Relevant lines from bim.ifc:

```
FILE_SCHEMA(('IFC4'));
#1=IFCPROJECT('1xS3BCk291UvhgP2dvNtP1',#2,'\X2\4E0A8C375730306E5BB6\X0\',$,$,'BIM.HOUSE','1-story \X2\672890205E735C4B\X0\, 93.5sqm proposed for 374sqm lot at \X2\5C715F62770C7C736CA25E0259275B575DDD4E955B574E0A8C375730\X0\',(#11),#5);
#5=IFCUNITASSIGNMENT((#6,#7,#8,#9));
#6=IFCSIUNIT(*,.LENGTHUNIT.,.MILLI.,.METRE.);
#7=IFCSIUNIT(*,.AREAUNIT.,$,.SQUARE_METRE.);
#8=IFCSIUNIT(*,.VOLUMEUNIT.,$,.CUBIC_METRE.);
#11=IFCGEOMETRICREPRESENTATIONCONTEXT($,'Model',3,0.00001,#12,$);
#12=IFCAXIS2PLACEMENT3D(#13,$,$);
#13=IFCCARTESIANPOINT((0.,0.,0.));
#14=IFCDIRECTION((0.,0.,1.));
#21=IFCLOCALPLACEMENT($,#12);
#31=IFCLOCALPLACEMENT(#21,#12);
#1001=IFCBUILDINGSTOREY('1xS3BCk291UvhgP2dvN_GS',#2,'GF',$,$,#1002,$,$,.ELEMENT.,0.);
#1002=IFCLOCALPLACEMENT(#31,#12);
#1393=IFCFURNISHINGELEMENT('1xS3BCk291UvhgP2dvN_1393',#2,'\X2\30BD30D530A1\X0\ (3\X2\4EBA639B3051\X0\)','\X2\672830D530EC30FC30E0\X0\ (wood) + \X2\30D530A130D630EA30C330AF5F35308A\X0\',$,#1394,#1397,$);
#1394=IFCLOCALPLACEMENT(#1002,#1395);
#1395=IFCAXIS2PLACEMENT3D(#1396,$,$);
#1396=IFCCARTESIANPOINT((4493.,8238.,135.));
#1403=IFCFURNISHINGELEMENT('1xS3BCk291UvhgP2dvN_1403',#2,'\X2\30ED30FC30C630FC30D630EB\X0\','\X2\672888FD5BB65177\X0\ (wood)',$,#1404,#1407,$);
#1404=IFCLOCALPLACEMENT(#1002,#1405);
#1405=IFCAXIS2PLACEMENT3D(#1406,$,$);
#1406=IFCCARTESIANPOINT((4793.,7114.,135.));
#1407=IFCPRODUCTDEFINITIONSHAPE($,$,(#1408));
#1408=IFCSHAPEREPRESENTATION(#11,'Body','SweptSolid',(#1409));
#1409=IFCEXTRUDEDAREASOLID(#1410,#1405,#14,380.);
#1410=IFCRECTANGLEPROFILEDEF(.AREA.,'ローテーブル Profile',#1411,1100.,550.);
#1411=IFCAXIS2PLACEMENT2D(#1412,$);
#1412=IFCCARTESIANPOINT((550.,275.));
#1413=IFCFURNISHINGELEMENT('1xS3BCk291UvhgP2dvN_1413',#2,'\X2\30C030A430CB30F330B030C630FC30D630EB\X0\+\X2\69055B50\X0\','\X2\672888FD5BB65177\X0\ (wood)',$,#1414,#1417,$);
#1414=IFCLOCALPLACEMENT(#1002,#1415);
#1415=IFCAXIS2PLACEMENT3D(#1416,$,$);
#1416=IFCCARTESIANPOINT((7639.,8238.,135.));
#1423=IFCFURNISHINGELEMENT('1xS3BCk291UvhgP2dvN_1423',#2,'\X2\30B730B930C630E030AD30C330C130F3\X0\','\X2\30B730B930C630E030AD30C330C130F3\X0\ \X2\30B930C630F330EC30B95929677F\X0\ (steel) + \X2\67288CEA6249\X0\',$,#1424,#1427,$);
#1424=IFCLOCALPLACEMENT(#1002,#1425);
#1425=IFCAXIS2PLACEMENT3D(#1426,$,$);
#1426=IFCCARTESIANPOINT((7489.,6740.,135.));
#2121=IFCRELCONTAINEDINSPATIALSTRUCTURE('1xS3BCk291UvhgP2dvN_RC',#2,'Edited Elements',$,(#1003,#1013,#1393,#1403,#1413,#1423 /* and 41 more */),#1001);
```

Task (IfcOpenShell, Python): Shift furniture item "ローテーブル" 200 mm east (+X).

```python
import ifcopenshell
import ifcopenshell.api.geometry
import ifcopenshell.util.placement
import ifcopenshell.util.unit

model = ifcopenshell.open("bim.ifc")
unit_scale = ifcopenshell.util.unit.calculate_unit_scale(model)

item = model.by_guid("1xS3BCk291UvhgP2dvN_1403")
matrix = ifcopenshell.util.placement.get_local_placement(item.ObjectPlacement)
matrix[0, 3] += 0.2 / unit_scale
ifcopenshell.api.geometry.edit_object_placement(model, product=item, matrix=matrix, is_si=False)

print(ifcopenshell.util.placement.get_local_placement(item.ObjectPlacement).round(3) + 0.0)

model.write("bim_edited.ifc")
```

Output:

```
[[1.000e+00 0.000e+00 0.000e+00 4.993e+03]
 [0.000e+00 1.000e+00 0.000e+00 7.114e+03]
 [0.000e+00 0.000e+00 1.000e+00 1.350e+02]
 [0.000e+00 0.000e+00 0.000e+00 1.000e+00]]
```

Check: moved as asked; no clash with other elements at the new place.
